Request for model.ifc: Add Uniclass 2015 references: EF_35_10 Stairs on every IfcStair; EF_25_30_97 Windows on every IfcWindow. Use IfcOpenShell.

First a look at what the model holds.

```python
import ifcopenshell

model = ifcopenshell.open("model.ifc")
print(model.schema)
print("classifications:", [c.Name for c in model.by_type("IfcClassification")])
for ifc_class in ("IfcDoor", "IfcRoof", "IfcStair", "IfcWall", "IfcWindow"):
    print(ifc_class, len(model.by_type(ifc_class)))
```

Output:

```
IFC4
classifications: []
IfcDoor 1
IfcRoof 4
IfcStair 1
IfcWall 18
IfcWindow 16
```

```python
import ifcopenshell
import ifcopenshell.api.classification

model = ifcopenshell.open("model.ifc")

system = ifcopenshell.api.classification.add_classification(model, classification="Uniclass 2015")

codes = {
    "IfcStair": ("EF_35_10", "Stairs"),
    "IfcWindow": ("EF_25_30_97", "Windows"),
}
for ifc_class, (code, name) in codes.items():
    products = model.by_type(ifc_class)
    ifcopenshell.api.classification.add_reference(
        model, products=products, classification=system, identification=code, name=name
    )
    print(code, len(products))

model.write("model_v2.ifc")
```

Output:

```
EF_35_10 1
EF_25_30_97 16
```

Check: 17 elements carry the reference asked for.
